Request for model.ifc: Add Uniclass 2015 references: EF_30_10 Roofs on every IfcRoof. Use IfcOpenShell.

First a look at what the model holds.

```python
import ifcopenshell

model = ifcopenshell.open("model.ifc")
print(model.schema)
print("classifications:", [c.Name for c in model.by_type("IfcClassification")])
for ifc_class in ("IfcDoor", "IfcRoof", "IfcStair", "IfcWall", "IfcWindow"):
    print(ifc_class, len(model.by_type(ifc_class)))
```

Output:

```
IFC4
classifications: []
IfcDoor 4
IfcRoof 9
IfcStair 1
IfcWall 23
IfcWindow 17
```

```python
import ifcopenshell
import ifcopenshell.api.classification

model = ifcopenshell.open("model.ifc")

system = ifcopenshell.api.classification.add_classification(model, classification="Uniclass 2015")

codes = {
    "IfcRoof": ("EF_30_10", "Roofs"),
}
for ifc_class, (code, name) in codes.items():
    products = model.by_type(ifc_class)
    ifcopenshell.api.classification.add_reference(
        model, products=products, classification=system, identification=code, name=name
    )
    print(code, len(products))

model.write("model_edited.ifc")
```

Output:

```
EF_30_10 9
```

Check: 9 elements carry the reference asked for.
